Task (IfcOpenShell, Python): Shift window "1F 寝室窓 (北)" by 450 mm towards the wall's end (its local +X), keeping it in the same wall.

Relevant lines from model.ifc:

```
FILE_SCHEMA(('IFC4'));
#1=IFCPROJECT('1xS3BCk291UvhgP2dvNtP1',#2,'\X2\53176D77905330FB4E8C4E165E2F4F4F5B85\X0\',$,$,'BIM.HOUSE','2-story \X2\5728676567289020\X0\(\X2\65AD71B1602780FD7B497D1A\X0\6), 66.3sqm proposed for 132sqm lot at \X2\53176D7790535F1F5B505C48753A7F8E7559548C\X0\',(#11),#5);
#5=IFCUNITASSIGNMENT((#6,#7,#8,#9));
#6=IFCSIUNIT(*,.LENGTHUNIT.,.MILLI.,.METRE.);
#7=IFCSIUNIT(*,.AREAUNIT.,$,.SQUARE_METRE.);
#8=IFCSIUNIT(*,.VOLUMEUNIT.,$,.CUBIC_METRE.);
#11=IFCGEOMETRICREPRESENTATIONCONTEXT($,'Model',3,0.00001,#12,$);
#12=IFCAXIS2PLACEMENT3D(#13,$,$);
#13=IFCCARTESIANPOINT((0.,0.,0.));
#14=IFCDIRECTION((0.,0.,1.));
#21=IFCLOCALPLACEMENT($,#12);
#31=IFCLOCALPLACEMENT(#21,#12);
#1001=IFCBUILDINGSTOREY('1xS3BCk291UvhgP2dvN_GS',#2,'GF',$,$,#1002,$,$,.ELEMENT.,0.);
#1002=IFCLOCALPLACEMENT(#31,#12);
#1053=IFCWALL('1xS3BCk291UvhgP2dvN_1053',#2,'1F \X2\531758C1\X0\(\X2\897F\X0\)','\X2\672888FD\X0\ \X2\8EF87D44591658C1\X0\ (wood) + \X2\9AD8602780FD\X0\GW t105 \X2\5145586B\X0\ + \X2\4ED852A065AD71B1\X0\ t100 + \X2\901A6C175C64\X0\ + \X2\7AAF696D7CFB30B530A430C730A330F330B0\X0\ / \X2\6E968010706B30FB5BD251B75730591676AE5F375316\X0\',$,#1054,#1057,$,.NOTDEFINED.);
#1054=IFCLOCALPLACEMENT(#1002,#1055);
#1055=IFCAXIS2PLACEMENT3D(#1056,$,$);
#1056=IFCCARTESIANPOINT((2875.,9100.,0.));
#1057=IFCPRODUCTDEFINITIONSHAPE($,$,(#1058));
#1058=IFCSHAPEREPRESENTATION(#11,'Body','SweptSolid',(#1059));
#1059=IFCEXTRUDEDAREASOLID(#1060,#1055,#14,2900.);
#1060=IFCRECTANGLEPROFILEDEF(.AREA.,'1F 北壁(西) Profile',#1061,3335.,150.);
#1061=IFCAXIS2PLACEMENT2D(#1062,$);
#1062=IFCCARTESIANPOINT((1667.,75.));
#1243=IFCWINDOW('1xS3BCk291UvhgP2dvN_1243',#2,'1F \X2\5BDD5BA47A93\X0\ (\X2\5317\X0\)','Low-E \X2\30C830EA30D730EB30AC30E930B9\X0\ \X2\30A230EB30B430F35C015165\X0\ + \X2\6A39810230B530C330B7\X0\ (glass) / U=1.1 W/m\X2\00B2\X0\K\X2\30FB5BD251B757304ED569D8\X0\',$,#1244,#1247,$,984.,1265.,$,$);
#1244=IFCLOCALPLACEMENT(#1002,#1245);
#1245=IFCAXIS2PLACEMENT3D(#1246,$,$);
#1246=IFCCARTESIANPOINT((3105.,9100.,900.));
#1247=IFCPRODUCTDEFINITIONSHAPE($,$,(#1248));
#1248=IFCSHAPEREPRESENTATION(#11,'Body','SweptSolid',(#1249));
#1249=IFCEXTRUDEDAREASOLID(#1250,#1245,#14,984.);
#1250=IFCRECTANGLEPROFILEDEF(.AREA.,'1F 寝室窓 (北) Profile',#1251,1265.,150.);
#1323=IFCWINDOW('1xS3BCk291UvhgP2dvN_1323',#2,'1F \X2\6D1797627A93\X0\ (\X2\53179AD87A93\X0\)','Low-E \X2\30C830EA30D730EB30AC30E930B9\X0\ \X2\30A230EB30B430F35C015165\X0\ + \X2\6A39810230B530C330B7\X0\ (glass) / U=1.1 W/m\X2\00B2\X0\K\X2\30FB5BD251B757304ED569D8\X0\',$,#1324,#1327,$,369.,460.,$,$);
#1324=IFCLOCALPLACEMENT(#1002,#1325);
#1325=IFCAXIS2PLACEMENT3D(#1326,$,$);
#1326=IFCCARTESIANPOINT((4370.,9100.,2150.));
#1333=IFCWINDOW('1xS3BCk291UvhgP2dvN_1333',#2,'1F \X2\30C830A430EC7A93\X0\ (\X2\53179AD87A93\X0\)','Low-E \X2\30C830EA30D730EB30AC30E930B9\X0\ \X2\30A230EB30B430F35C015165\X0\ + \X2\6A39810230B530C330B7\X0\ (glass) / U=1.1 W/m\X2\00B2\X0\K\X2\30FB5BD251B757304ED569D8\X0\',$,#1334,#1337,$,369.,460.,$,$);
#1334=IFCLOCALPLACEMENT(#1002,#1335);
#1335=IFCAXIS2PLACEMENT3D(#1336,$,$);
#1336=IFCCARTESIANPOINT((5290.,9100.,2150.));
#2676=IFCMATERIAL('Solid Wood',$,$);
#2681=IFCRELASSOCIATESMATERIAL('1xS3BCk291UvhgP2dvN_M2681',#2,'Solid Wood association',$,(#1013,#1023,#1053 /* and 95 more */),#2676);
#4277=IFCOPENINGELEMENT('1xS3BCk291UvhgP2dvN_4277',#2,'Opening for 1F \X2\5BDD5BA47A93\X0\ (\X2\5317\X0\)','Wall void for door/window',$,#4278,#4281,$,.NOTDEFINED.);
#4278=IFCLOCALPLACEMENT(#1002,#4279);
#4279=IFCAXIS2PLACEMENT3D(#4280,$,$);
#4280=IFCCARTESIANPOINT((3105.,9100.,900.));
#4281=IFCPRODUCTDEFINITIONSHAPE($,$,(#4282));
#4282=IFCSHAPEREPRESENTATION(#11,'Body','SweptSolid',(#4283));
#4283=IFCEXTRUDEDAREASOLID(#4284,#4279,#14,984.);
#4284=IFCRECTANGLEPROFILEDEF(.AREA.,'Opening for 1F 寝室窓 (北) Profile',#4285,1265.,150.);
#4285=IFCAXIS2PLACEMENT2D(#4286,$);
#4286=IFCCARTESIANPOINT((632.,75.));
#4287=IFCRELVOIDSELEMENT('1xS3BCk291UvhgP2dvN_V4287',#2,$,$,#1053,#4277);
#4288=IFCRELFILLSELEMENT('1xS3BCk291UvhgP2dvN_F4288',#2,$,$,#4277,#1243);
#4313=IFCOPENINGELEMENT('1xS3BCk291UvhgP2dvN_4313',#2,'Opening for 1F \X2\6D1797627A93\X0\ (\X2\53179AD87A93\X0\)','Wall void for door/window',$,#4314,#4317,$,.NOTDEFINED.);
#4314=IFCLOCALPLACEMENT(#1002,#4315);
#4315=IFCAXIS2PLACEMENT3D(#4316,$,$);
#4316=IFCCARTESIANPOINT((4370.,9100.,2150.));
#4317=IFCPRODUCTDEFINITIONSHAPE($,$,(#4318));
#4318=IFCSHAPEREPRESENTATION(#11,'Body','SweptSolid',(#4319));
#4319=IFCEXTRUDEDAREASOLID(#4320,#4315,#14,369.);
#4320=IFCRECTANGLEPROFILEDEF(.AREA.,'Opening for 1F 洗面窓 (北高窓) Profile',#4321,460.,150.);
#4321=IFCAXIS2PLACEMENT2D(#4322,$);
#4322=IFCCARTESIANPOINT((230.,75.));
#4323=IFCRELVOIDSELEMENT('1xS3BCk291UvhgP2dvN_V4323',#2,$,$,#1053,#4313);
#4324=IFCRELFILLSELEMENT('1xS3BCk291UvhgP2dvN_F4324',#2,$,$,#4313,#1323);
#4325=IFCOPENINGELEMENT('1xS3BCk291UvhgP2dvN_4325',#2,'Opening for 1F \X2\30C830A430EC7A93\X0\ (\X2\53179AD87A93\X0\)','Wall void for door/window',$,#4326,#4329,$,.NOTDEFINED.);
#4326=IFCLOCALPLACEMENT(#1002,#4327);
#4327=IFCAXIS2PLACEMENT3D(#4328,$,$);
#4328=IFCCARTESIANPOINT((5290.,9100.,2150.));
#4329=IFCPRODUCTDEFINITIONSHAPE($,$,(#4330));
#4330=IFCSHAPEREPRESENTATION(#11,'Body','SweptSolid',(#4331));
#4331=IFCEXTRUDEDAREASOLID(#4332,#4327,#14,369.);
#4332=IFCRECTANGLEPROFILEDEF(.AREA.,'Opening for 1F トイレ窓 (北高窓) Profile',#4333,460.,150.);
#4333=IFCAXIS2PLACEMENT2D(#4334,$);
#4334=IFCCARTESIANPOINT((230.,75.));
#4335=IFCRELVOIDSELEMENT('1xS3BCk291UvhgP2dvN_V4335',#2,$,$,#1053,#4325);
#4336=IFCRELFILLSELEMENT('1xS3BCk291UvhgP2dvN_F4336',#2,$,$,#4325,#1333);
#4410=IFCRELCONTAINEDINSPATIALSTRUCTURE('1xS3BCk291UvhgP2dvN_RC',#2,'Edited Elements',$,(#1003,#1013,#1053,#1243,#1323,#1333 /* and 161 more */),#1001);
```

```python
import ifcopenshell
import ifcopenshell.api.geometry
import ifcopenshell.util.placement
import ifcopenshell.util.unit

model = ifcopenshell.open("model.ifc")
unit_scale = ifcopenshell.util.unit.calculate_unit_scale(model)

window = model.by_id(1243)
opening = window.FillsVoids[0].RelatingOpeningElement
wall = opening.VoidsElements[0].RelatingBuildingElement

wall_matrix = ifcopenshell.util.placement.get_local_placement(wall.ObjectPlacement)
shift = wall_matrix[:3, 0] * 0.45 / unit_scale
before = ifcopenshell.util.placement.get_local_placement(window.ObjectPlacement)[:3, 3].copy()

# The window is not placed relative to its opening, so move both.
for product in (opening, window):
    matrix = ifcopenshell.util.placement.get_local_placement(product.ObjectPlacement)
    matrix[:3, 3] += shift
    ifcopenshell.api.geometry.edit_object_placement(model, product=product, matrix=matrix, is_si=False)

after = ifcopenshell.util.placement.get_local_placement(window.ObjectPlacement)[:3, 3]
print("window moved by", (after - before).round(3) + 0.0)

model.write("model_v2.ifc")
```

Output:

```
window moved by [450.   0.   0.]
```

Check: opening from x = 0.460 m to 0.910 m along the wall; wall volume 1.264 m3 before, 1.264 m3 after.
